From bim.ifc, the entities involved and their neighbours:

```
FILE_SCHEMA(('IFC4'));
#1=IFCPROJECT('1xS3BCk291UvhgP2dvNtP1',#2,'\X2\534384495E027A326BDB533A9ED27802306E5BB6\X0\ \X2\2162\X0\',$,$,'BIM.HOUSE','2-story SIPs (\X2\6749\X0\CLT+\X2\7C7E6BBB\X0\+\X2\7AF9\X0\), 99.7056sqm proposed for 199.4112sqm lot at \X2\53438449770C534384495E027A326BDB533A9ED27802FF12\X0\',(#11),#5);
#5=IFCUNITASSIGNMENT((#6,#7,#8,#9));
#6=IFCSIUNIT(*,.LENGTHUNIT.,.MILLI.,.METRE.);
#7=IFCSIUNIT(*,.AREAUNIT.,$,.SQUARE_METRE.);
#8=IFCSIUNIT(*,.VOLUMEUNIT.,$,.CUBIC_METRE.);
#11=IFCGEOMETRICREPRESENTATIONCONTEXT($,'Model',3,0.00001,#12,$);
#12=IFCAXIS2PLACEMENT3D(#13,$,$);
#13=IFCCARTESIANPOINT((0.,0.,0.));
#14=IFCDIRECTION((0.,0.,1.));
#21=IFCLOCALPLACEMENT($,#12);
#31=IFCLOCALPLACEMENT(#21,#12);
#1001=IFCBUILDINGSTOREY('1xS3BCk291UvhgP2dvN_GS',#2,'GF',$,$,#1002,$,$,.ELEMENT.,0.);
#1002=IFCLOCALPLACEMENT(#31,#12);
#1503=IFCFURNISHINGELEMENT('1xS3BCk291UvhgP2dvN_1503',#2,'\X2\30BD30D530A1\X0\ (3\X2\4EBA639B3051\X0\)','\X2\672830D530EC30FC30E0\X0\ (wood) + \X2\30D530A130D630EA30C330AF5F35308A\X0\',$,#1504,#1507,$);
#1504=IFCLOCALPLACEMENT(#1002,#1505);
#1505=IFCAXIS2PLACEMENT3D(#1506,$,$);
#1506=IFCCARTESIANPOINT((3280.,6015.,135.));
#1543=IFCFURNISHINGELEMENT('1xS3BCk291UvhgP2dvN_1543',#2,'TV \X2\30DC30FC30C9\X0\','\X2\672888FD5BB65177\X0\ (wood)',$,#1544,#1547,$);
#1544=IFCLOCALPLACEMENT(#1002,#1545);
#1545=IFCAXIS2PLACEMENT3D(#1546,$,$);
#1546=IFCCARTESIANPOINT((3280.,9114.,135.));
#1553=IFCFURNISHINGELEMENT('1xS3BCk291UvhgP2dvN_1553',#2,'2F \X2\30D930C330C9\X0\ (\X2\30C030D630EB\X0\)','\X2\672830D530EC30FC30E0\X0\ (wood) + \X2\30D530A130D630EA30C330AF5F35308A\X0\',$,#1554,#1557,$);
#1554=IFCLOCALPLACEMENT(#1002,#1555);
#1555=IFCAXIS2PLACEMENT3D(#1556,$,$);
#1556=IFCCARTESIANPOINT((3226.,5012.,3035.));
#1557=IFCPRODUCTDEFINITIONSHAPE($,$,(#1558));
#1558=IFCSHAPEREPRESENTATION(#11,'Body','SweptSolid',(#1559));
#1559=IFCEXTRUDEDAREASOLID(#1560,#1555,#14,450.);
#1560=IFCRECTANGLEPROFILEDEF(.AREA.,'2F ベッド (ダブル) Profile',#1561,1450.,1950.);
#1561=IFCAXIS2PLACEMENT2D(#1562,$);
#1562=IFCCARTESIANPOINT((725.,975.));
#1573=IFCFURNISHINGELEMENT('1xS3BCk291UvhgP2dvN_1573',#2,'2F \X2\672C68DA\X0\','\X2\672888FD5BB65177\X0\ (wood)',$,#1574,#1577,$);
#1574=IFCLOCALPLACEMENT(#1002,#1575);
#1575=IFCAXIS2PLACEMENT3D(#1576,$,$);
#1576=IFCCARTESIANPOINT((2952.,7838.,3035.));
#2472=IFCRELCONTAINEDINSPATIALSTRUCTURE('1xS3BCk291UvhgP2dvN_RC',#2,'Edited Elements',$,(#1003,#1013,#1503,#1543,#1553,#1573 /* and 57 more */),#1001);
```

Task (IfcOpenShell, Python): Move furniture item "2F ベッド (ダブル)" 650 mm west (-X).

```python
import ifcopenshell
import ifcopenshell.api.geometry
import ifcopenshell.util.placement
import ifcopenshell.util.unit

model = ifcopenshell.open("bim.ifc")
unit_scale = ifcopenshell.util.unit.calculate_unit_scale(model)

item = model.by_id(1553)
matrix = ifcopenshell.util.placement.get_local_placement(item.ObjectPlacement)
matrix[0, 3] -= 0.65 / unit_scale
ifcopenshell.api.geometry.edit_object_placement(model, product=item, matrix=matrix, is_si=False)

print(ifcopenshell.util.placement.get_local_placement(item.ObjectPlacement).round(3) + 0.0)

model.write("bim-out.ifc")
```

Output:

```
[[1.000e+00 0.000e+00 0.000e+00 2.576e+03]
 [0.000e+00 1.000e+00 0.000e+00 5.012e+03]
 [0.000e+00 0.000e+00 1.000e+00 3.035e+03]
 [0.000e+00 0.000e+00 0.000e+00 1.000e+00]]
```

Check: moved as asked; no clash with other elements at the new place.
